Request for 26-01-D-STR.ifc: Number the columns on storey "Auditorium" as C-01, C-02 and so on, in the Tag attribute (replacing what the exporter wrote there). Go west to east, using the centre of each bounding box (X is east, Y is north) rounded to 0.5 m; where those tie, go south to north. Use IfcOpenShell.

First a look at what the model holds.

```python
import ifcopenshell
import ifcopenshell.util.element
import ifcopenshell.util.placement

model = ifcopenshell.open("26-01-D-STR.ifc")
print(model.schema)
storey = next(s for s in model.by_type("IfcBuildingStorey") if s.Name == "Auditorium")
columns = [e for e in ifcopenshell.util.element.get_decomposition(storey) if e.is_a("IfcColumn")]
for e in sorted(columns, key=lambda e: e.id()):
    origin = ifcopenshell.util.placement.get_local_placement(e.ObjectPlacement)[:3, 3]
    print(e.id(), e.Tag, e.Name, origin.round(2) + 0.0, sep=" | ")
```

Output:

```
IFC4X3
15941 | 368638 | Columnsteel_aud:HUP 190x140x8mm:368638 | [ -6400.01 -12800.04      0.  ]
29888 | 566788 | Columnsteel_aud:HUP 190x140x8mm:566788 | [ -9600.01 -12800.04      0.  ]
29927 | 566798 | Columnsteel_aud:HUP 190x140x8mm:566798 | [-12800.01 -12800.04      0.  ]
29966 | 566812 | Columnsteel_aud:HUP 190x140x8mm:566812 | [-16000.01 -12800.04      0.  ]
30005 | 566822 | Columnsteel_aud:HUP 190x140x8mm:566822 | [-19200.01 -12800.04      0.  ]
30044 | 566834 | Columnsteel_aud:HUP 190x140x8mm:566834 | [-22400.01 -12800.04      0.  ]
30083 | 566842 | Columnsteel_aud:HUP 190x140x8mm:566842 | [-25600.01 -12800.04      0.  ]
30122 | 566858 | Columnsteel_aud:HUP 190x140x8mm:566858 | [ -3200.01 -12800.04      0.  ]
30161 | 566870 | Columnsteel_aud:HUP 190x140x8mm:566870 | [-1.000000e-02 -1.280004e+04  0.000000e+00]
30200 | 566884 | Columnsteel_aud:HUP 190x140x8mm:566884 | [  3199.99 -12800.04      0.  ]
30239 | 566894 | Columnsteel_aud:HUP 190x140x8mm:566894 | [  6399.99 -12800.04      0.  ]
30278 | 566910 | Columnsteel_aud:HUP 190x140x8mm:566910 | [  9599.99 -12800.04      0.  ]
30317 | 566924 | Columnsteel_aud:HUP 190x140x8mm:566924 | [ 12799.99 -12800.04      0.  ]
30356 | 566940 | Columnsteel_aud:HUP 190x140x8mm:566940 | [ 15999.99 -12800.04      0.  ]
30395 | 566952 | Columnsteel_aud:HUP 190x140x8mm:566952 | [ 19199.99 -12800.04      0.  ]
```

```python
import ifcopenshell
import ifcopenshell.geom
import ifcopenshell.util.element
import ifcopenshell.util.shape

model = ifcopenshell.open("26-01-D-STR.ifc")
settings = ifcopenshell.geom.settings()
settings.set("use-world-coords", True)


def centre(element):
    shape = ifcopenshell.geom.create_shape(settings, element)
    return ifcopenshell.util.shape.get_bbox_centroid(shape.geometry)


storey = next(s for s in model.by_type("IfcBuildingStorey") if s.Name == "Auditorium")
columns = [e for e in ifcopenshell.util.element.get_decomposition(storey) if e.is_a("IfcColumn")]

# Insertion points can sit at a corner or the storey origin, so sort by the geometry (in metres).
centres = {e: centre(e) for e in columns}
columns.sort(key=lambda e: (round(centres[e][0] / 0.5), centres[e][1]))

for i, e in enumerate(columns, start=1):
    number = f"C-{i:02d}"
    e.Tag = number
    print(e.id(), number)

model.write("26-01-D-STR_rev.ifc")
```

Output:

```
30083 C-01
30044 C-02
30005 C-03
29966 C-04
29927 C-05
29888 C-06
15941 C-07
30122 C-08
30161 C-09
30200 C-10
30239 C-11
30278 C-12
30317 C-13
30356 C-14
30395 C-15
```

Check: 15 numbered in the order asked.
